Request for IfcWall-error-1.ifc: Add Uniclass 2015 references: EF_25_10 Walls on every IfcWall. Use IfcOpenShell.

First a look at what the model holds.

```python
import ifcopenshell

model = ifcopenshell.open("IfcWall-error-1.ifc")
print(model.schema)
print("classifications:", [c.Name for c in model.by_type("IfcClassification")])
for ifc_class in ("IfcDoor", "IfcRoof", "IfcStair", "IfcWall", "IfcWindow"):
    print(ifc_class, len(model.by_type(ifc_class)))
```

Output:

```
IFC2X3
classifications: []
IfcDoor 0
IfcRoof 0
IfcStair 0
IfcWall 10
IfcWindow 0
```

```python
import ifcopenshell
import ifcopenshell.api.classification

model = ifcopenshell.open("IfcWall-error-1.ifc")

# IFC2X3 requires Source and Edition and has no link from the project to the system.
system = model.create_entity("IfcClassification", Source="NBS", Edition="2015", Name="Uniclass 2015")

codes = {
    "IfcWall": ("EF_25_10", "Walls"),
}
for ifc_class, (code, name) in codes.items():
    products = model.by_type(ifc_class)
    ifcopenshell.api.classification.add_reference(
        model, products=products, classification=system, identification=code, name=name
    )
    print(code, len(products))

model.write("IfcWall-error-1_edited.ifc")
```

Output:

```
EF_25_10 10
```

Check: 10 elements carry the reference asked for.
